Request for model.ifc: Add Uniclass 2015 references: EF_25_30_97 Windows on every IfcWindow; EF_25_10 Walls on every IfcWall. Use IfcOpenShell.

First a look at what the model holds.

```python
import ifcopenshell

model = ifcopenshell.open("model.ifc")
print(model.schema)
print("classifications:", [c.Name for c in model.by_type("IfcClassification")])
for ifc_class in ("IfcDoor", "IfcRoof", "IfcStair", "IfcWall", "IfcWindow"):
    print(ifc_class, len(model.by_type(ifc_class)))
```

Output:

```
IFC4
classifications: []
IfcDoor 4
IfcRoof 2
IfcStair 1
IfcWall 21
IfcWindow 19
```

```python
import ifcopenshell
import ifcopenshell.api.classification

model = ifcopenshell.open("model.ifc")

system = ifcopenshell.api.classification.add_classification(model, classification="Uniclass 2015")

codes = {
    "IfcWindow": ("EF_25_30_97", "Windows"),
    "IfcWall": ("EF_25_10", "Walls"),
}
for ifc_class, (code, name) in codes.items():
    products = model.by_type(ifc_class)
    ifcopenshell.api.classification.add_reference(
        model, products=products, classification=system, identification=code, name=name
    )
    print(code, len(products))

model.write("model_updated.ifc")
```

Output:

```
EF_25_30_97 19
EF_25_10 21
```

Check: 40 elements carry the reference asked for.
